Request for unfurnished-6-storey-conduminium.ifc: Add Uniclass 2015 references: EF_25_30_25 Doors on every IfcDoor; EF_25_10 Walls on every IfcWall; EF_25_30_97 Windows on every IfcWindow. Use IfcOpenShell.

First a look at what the model holds.

```python
import ifcopenshell

model = ifcopenshell.open("unfurnished-6-storey-conduminium.ifc")
print(model.schema)
print("classifications:", [c.Name for c in model.by_type("IfcClassification")])
for ifc_class in ("IfcDoor", "IfcRoof", "IfcStair", "IfcWall", "IfcWindow"):
    print(ifc_class, len(model.by_type(ifc_class)))
```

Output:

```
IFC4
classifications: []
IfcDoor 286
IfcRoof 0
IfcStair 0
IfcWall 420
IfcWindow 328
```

```python
import ifcopenshell
import ifcopenshell.api.classification

model = ifcopenshell.open("unfurnished-6-storey-conduminium.ifc")

system = ifcopenshell.api.classification.add_classification(model, classification="Uniclass 2015")

codes = {
    "IfcDoor": ("EF_25_30_25", "Doors"),
    "IfcWall": ("EF_25_10", "Walls"),
    "IfcWindow": ("EF_25_30_97", "Windows"),
}
for ifc_class, (code, name) in codes.items():
    products = model.by_type(ifc_class)
    ifcopenshell.api.classification.add_reference(
        model, products=products, classification=system, identification=code, name=name
    )
    print(code, len(products))

model.write("unfurnished-6-storey-conduminium_updated.ifc")
```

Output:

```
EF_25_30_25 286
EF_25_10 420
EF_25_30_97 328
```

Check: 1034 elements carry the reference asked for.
